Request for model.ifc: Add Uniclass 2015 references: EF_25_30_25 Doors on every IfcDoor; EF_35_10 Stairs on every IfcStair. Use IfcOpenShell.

First a look at what the model holds.

```python
import ifcopenshell

model = ifcopenshell.open("model.ifc")
print(model.schema)
print("classifications:", [c.Name for c in model.by_type("IfcClassification")])
for ifc_class in ("IfcDoor", "IfcRoof", "IfcStair", "IfcWall", "IfcWindow"):
    print(ifc_class, len(model.by_type(ifc_class)))
```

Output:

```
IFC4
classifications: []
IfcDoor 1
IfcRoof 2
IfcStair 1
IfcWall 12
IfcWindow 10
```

```python
import ifcopenshell
import ifcopenshell.api.classification

model = ifcopenshell.open("model.ifc")

system = ifcopenshell.api.classification.add_classification(model, classification="Uniclass 2015")

codes = {
    "IfcDoor": ("EF_25_30_25", "Doors"),
    "IfcStair": ("EF_35_10", "Stairs"),
}
for ifc_class, (code, name) in codes.items():
    products = model.by_type(ifc_class)
    ifcopenshell.api.classification.add_reference(
        model, products=products, classification=system, identification=code, name=name
    )
    print(code, len(products))

model.write("model_rev.ifc")
```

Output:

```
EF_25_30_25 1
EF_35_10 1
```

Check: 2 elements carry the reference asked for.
